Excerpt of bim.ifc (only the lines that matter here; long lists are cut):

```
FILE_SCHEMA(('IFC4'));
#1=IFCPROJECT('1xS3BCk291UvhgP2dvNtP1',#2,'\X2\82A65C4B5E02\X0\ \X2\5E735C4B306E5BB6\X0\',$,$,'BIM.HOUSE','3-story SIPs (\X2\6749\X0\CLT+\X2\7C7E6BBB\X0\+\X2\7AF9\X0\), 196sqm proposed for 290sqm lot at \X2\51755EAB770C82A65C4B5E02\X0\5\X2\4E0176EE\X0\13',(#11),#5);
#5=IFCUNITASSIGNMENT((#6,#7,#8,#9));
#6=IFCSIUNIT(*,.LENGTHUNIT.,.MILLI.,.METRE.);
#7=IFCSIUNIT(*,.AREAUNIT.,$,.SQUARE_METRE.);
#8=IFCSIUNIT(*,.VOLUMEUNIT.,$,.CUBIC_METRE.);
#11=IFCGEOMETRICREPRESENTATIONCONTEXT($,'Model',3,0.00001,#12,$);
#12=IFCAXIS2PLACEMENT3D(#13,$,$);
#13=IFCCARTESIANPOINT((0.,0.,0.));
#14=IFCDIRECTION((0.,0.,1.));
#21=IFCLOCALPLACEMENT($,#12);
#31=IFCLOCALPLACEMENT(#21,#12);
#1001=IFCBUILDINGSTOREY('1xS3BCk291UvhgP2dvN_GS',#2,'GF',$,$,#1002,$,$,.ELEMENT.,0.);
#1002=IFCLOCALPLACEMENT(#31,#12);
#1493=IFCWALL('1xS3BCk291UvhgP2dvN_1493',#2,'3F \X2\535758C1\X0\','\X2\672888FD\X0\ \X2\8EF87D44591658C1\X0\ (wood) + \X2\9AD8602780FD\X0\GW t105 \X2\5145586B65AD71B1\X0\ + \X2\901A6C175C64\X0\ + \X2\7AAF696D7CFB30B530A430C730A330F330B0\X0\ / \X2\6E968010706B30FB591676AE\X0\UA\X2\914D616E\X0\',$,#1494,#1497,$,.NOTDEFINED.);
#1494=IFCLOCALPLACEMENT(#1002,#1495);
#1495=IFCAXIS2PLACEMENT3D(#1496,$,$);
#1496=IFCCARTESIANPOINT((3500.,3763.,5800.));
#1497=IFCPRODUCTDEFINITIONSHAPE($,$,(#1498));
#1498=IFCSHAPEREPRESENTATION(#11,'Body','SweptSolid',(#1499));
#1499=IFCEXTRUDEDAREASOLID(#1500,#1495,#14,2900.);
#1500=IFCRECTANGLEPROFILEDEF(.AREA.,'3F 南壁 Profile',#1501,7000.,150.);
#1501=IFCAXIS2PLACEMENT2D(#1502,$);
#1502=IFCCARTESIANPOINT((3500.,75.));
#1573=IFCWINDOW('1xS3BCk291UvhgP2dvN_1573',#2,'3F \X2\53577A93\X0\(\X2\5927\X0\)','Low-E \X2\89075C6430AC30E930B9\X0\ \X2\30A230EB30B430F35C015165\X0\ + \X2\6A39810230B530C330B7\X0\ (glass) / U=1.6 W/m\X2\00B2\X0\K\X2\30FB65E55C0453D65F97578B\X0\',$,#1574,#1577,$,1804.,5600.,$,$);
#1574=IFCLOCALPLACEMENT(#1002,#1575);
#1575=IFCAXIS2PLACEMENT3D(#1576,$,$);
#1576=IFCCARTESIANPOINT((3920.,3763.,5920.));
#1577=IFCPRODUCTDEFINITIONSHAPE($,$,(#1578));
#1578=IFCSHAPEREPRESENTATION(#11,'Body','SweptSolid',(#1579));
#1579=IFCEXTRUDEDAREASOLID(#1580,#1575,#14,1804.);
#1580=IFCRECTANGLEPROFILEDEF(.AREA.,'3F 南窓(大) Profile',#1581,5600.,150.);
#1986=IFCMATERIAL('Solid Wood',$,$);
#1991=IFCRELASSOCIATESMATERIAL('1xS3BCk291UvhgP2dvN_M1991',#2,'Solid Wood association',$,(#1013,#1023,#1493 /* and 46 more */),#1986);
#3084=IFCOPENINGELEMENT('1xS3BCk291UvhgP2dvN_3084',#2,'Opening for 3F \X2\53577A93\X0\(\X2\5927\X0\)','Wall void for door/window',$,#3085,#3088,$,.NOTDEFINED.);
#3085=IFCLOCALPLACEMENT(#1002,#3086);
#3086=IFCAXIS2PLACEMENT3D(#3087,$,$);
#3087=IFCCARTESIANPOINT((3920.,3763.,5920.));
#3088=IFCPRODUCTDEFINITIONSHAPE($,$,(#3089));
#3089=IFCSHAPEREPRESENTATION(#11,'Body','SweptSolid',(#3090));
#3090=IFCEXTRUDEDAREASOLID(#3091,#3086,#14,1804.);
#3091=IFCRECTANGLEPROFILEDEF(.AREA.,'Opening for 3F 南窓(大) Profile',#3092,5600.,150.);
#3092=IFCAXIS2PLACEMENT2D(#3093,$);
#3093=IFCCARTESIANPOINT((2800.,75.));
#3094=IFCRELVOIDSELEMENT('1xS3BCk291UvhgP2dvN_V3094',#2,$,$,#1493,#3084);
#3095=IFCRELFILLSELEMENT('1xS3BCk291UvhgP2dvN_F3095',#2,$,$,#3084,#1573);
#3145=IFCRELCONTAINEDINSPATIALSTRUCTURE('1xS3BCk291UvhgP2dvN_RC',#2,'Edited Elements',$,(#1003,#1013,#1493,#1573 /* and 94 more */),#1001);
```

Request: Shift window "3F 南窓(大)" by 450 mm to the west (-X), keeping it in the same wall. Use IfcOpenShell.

```python
import ifcopenshell
import ifcopenshell.api.geometry
import ifcopenshell.util.placement

model = ifcopenshell.open("bim.ifc")

window = model.by_guid("1xS3BCk291UvhgP2dvN_1573")
opening = window.FillsVoids[0].RelatingOpeningElement
wall = opening.VoidsElements[0].RelatingBuildingElement

wall_matrix = ifcopenshell.util.placement.get_local_placement(wall.ObjectPlacement)
shift = wall_matrix[:3, 0] * -450.0
before = ifcopenshell.util.placement.get_local_placement(window.ObjectPlacement)[:3, 3].copy()

# The window is not placed relative to its opening, so move both.
for product in (opening, window):
    matrix = ifcopenshell.util.placement.get_local_placement(product.ObjectPlacement)
    matrix[:3, 3] += shift
    ifcopenshell.api.geometry.edit_object_placement(model, product=product, matrix=matrix, is_si=False)

after = ifcopenshell.util.placement.get_local_placement(window.ObjectPlacement)[:3, 3]
print("window moved by", (after - before).round(3) + 0.0)

model.write("bim_edited.ifc")
```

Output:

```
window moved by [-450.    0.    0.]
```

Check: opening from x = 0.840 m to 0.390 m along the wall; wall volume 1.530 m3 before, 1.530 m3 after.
